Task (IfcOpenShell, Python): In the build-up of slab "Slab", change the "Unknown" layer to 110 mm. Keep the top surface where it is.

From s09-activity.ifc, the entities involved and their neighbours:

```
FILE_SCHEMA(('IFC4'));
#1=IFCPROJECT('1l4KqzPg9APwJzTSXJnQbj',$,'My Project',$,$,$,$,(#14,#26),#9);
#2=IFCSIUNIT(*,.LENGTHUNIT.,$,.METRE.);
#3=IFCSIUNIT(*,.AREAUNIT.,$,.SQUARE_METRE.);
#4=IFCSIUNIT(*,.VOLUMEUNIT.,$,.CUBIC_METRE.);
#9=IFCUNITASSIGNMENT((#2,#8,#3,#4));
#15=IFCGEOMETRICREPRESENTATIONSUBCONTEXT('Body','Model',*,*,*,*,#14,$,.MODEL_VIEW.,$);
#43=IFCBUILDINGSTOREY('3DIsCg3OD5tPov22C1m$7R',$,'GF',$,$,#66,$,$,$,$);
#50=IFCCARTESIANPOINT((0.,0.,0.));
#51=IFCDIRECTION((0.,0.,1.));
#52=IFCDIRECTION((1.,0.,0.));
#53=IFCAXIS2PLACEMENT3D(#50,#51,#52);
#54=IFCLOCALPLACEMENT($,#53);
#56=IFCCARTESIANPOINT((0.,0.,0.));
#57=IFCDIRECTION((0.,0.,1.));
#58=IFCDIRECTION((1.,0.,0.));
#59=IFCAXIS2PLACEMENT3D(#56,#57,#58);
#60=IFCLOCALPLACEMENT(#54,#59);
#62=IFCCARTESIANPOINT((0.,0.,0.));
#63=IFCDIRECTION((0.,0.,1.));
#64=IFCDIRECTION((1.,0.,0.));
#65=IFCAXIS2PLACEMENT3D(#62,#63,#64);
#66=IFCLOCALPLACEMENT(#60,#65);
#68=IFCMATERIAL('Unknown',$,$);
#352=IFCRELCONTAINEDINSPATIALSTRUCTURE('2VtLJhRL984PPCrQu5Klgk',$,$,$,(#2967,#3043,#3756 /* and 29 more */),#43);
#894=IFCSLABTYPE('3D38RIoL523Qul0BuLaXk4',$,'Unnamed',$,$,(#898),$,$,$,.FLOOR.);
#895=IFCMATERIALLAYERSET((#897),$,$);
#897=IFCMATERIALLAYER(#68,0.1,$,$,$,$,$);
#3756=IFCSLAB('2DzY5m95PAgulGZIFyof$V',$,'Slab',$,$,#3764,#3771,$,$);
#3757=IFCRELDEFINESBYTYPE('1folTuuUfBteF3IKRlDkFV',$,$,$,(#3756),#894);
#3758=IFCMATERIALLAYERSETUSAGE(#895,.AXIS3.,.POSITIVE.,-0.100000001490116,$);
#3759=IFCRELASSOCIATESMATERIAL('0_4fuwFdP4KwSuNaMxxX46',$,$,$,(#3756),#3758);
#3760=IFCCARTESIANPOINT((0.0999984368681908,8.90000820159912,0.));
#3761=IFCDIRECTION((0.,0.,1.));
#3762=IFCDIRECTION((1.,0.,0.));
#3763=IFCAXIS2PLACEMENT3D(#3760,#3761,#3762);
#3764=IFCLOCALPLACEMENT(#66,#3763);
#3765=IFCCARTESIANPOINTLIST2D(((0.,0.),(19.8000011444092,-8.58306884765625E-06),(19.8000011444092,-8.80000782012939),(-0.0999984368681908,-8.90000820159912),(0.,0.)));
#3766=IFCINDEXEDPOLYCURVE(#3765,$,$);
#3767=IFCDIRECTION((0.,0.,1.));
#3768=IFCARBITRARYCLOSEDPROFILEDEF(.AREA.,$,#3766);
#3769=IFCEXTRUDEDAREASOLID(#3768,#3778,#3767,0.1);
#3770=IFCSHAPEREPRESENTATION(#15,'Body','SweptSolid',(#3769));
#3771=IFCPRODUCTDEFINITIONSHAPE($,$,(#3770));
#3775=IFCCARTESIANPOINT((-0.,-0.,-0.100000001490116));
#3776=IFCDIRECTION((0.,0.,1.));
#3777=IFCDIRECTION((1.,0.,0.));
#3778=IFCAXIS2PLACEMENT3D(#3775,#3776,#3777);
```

```python
import ifcopenshell
import ifcopenshell.util.element
import ifcopenshell.util.representation
import ifcopenshell.util.unit

model = ifcopenshell.open("s09-activity.ifc")
unit_scale = ifcopenshell.util.unit.calculate_unit_scale(model)

layer_set = model.by_id(895)
layer = next(l for l in layer_set.MaterialLayers if l.Material and l.Material.Name == "Unknown")
change = 0.11 / unit_scale - layer.LayerThickness
layer.LayerThickness += change

# Geometry does not follow the layer set by itself.
slabs = [e for e in ifcopenshell.util.element.get_elements_by_material(model, layer_set) if e.is_a("IfcSlab")]
for slab in sorted(slabs, key=lambda e: e.id()):
    body = ifcopenshell.util.representation.get_representation(slab, "Model", "Body")
    solid = body.Items[0]
    old_depth = solid.Depth
    solid.Depth += change
    # Extruded upwards: lower the start of the extrusion so the top stays.
    x, y, z = solid.Position.Location.Coordinates
    solid.Position.Location = model.createIfcCartesianPoint((x, y, z - change))
    print(slab.id(), f"{old_depth:g} -> {solid.Depth:g}")

# The layers are counted up from the underside, which has moved.
for usage in {ifcopenshell.util.element.get_material(slab) for slab in slabs}:
    usage.OffsetFromReferenceLine -= change

model.write("s09-activity_rev.ifc")
```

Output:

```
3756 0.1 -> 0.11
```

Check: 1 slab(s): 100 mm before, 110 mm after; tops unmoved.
